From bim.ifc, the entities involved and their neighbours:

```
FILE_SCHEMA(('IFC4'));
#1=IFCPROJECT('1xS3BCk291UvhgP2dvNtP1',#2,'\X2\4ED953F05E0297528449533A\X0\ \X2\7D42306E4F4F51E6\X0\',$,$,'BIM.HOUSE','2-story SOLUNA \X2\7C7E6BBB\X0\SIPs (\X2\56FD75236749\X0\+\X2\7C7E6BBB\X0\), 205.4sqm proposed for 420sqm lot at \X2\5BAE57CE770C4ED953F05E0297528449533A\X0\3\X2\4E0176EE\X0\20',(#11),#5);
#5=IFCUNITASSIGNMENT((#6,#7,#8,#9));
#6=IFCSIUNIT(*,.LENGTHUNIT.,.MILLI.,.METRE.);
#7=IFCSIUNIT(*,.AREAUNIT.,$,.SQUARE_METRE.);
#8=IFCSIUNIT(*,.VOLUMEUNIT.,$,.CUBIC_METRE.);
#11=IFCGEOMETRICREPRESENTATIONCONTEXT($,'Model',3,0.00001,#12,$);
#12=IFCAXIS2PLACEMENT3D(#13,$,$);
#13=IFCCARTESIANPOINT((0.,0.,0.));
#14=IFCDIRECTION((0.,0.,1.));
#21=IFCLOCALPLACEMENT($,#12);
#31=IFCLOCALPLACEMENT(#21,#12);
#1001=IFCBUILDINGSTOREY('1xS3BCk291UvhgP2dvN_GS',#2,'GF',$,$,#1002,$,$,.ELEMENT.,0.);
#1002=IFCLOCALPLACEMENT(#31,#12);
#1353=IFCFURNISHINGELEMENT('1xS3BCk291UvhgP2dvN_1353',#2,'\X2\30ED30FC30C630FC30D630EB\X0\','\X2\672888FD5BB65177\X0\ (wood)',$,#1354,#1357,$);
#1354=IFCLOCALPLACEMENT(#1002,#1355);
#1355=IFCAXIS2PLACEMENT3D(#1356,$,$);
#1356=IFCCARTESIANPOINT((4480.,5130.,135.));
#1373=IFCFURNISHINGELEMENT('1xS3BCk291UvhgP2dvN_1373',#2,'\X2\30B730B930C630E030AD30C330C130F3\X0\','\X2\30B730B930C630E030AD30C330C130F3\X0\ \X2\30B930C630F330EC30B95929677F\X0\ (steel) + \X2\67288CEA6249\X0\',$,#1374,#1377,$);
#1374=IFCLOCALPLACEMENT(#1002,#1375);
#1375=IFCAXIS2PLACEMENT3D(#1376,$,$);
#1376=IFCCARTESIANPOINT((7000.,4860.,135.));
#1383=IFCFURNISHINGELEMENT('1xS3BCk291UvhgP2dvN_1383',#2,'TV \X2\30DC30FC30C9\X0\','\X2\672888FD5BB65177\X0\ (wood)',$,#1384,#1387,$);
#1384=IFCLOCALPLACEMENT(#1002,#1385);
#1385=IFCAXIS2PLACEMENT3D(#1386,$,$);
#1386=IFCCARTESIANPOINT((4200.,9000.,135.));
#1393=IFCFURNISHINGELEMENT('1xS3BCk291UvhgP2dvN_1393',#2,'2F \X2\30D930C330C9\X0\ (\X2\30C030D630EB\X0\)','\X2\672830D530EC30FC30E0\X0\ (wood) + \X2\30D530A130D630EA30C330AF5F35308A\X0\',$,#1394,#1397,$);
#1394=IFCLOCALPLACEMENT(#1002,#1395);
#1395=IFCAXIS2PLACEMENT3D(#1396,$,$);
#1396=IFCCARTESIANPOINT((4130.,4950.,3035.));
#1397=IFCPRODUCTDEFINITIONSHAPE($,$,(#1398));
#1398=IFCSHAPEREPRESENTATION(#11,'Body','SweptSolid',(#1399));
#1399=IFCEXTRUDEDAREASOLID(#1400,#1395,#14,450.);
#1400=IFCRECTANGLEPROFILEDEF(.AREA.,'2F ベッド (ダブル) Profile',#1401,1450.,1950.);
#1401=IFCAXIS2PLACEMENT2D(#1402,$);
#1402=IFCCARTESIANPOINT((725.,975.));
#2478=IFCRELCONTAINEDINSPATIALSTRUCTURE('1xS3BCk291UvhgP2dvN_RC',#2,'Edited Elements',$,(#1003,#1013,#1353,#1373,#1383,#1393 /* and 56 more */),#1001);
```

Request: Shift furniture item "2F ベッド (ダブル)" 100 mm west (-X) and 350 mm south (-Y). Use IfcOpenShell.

```python
import ifcopenshell
import ifcopenshell.api.geometry
import ifcopenshell.util.placement
import ifcopenshell.util.unit

model = ifcopenshell.open("bim.ifc")
unit_scale = ifcopenshell.util.unit.calculate_unit_scale(model)

item = model.by_guid("1xS3BCk291UvhgP2dvN_1393")
matrix = ifcopenshell.util.placement.get_local_placement(item.ObjectPlacement)
matrix[0, 3] -= 0.1 / unit_scale
matrix[1, 3] -= 0.35 / unit_scale
ifcopenshell.api.geometry.edit_object_placement(model, product=item, matrix=matrix, is_si=False)

print(ifcopenshell.util.placement.get_local_placement(item.ObjectPlacement).round(3) + 0.0)

model.write("bim_edited.ifc")
```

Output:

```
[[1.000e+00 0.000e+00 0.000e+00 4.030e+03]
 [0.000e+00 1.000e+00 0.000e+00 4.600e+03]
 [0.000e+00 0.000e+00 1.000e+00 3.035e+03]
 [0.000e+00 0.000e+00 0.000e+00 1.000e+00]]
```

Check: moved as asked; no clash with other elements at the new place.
